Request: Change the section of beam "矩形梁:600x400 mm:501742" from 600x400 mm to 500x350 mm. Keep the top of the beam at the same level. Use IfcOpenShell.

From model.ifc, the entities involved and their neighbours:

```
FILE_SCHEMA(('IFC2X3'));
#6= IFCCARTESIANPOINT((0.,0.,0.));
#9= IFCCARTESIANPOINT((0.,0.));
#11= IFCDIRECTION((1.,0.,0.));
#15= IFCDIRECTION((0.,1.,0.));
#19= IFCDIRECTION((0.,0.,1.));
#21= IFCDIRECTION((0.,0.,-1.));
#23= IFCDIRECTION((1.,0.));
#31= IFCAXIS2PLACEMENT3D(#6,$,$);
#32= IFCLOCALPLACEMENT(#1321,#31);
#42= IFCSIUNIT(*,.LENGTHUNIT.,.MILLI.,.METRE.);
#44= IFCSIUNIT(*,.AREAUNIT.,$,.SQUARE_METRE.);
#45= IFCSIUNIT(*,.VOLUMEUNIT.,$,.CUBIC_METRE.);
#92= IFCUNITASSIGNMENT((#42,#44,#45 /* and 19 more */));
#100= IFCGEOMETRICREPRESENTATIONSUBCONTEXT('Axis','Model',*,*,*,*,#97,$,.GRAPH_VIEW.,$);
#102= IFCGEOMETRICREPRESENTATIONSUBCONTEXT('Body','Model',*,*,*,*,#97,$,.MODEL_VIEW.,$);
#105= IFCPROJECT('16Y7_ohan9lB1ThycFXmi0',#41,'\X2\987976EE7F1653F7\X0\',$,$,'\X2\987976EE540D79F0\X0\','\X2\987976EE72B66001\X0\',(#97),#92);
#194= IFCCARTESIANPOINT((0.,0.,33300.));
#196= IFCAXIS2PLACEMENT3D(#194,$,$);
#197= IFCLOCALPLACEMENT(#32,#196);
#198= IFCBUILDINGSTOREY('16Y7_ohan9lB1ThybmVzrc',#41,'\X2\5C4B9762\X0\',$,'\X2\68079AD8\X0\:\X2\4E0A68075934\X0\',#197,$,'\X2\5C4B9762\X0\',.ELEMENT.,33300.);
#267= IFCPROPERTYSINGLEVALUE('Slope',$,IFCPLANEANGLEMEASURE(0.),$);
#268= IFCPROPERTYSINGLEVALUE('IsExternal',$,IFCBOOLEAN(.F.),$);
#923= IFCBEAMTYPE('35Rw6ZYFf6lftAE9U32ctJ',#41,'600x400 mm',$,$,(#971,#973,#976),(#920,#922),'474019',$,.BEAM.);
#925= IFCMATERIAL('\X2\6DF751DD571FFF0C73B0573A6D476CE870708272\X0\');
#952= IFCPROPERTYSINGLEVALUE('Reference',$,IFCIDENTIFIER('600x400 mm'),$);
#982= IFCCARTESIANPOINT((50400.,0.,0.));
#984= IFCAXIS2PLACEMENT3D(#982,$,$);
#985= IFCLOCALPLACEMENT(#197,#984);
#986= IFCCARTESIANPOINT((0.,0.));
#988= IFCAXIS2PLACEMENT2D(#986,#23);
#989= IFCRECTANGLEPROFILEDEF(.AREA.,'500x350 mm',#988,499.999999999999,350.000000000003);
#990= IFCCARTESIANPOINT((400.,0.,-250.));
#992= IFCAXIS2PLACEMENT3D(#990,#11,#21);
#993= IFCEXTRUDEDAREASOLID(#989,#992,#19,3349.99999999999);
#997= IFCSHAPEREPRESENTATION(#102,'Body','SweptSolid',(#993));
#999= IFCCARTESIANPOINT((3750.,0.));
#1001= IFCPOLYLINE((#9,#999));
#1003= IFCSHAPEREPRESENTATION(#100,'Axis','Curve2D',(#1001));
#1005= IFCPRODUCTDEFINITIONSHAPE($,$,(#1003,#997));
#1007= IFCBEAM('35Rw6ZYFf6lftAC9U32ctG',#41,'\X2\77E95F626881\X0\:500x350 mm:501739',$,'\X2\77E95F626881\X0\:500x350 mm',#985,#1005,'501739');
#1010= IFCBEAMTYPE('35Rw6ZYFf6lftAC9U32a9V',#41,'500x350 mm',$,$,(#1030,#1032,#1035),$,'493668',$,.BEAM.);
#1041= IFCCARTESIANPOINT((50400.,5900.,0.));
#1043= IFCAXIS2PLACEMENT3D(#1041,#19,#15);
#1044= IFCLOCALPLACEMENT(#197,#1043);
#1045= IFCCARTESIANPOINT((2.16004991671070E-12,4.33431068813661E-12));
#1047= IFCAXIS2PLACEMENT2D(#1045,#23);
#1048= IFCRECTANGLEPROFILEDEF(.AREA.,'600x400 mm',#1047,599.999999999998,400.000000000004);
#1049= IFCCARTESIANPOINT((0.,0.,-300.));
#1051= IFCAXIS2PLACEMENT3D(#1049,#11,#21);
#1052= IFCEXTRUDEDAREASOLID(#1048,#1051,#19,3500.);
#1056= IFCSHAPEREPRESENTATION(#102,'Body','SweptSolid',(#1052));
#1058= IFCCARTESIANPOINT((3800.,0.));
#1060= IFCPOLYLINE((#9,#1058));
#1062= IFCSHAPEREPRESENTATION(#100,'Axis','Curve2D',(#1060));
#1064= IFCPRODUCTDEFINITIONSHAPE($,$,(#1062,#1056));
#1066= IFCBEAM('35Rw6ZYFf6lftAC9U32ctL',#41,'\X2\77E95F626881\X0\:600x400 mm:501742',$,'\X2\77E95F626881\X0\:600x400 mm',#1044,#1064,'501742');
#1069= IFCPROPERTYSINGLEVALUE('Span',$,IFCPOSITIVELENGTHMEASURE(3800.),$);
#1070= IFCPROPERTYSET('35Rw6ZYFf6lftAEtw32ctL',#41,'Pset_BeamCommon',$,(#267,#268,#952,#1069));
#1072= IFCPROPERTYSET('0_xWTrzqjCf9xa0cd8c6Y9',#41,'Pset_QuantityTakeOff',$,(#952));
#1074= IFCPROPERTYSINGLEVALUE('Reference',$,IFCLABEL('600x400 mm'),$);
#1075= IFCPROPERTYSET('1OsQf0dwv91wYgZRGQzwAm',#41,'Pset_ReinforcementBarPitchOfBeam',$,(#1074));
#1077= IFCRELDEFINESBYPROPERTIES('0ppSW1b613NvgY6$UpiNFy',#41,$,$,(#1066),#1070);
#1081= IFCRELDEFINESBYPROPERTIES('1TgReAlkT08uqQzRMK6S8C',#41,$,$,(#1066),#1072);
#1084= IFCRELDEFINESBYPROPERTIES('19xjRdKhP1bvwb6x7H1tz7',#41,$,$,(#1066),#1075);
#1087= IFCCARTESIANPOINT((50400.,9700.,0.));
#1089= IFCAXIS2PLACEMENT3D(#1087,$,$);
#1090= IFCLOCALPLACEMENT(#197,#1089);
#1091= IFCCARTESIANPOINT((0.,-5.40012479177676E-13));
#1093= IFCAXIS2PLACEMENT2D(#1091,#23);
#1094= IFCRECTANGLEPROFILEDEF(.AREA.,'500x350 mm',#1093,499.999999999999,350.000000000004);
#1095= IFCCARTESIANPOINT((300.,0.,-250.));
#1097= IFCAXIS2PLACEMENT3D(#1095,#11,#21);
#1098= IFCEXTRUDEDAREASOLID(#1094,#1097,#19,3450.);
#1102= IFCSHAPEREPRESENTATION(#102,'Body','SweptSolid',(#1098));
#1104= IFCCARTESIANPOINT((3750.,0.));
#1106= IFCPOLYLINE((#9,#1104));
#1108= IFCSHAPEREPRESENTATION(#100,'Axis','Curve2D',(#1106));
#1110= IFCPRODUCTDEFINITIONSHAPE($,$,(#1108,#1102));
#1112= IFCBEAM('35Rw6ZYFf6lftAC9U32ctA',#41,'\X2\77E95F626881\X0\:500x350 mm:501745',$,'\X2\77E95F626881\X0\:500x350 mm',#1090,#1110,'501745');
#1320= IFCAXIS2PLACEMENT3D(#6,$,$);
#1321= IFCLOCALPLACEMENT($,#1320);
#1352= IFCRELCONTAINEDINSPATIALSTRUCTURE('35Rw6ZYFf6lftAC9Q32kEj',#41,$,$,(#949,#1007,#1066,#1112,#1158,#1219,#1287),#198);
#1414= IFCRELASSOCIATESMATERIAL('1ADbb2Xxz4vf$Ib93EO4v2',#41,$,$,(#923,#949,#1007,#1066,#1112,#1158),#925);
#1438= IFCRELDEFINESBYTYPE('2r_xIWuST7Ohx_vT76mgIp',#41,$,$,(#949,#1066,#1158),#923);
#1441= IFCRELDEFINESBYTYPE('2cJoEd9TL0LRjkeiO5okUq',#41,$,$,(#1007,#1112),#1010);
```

```python
import ifcopenshell
import ifcopenshell.api.pset
import ifcopenshell.api.type
import ifcopenshell.util.element
import ifcopenshell.util.representation

model = ifcopenshell.open("model.ifc")

member = model.by_guid("35Rw6ZYFf6lftAC9U32ctL")
source = next(p for p in model.by_type("IfcRectangleProfileDef") if p.ProfileName == "500x350 mm")

body = ifcopenshell.util.representation.get_representation(member, "Model", "Body")
solid = body.Items[0]
old_profile = solid.SweptArea

# Copy the section's sizes but keep this member's own profile position.
profile = ifcopenshell.util.element.copy(model, source)
# Profiles are centred, so shift by half the change in depth to hold the top.
shift = (old_profile.XDim - profile.XDim) / 2
x, y = old_profile.Position.Location.Coordinates
up = (-1.0, 0.0)  # upwards, in the solid's own plane
location = model.createIfcCartesianPoint((x + up[0] * shift, y + up[1] * shift))
profile.Position = model.createIfcAxis2Placement2D(location, old_profile.Position.RefDirection)
solid.SweptArea = profile
if not model.get_total_inverses(old_profile):
    ifcopenshell.util.element.remove_deep2(model, old_profile)

new_type = model.by_guid("35Rw6ZYFf6lftAC9U32a9V")
ifcopenshell.api.type.assign_type(
    model, related_objects=[member], relating_type=new_type, should_map_representations=False
)
member.Name = member.Name.replace("600x400 mm", "500x350 mm")
member.ObjectType = "矩形梁:500x350 mm"
pset = model.by_id(ifcopenshell.util.element.get_pset(member, "Pset_BeamCommon", should_inherit=False)["id"])
ifcopenshell.api.pset.edit_pset(model, pset=pset, properties={"Reference": "500x350 mm"})
pset = model.by_id(ifcopenshell.util.element.get_pset(member, "Pset_QuantityTakeOff", should_inherit=False)["id"])
ifcopenshell.api.pset.edit_pset(model, pset=pset, properties={"Reference": "500x350 mm"})
pset = model.by_id(ifcopenshell.util.element.get_pset(member, "Pset_ReinforcementBarPitchOfBeam", should_inherit=False)["id"])
ifcopenshell.api.pset.edit_pset(model, pset=pset, properties={"Reference": "500x350 mm"})

print(solid.SweptArea)

model.write("model_v2.ifc")
```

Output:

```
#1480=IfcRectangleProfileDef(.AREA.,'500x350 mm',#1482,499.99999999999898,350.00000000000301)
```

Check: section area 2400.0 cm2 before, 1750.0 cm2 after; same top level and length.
